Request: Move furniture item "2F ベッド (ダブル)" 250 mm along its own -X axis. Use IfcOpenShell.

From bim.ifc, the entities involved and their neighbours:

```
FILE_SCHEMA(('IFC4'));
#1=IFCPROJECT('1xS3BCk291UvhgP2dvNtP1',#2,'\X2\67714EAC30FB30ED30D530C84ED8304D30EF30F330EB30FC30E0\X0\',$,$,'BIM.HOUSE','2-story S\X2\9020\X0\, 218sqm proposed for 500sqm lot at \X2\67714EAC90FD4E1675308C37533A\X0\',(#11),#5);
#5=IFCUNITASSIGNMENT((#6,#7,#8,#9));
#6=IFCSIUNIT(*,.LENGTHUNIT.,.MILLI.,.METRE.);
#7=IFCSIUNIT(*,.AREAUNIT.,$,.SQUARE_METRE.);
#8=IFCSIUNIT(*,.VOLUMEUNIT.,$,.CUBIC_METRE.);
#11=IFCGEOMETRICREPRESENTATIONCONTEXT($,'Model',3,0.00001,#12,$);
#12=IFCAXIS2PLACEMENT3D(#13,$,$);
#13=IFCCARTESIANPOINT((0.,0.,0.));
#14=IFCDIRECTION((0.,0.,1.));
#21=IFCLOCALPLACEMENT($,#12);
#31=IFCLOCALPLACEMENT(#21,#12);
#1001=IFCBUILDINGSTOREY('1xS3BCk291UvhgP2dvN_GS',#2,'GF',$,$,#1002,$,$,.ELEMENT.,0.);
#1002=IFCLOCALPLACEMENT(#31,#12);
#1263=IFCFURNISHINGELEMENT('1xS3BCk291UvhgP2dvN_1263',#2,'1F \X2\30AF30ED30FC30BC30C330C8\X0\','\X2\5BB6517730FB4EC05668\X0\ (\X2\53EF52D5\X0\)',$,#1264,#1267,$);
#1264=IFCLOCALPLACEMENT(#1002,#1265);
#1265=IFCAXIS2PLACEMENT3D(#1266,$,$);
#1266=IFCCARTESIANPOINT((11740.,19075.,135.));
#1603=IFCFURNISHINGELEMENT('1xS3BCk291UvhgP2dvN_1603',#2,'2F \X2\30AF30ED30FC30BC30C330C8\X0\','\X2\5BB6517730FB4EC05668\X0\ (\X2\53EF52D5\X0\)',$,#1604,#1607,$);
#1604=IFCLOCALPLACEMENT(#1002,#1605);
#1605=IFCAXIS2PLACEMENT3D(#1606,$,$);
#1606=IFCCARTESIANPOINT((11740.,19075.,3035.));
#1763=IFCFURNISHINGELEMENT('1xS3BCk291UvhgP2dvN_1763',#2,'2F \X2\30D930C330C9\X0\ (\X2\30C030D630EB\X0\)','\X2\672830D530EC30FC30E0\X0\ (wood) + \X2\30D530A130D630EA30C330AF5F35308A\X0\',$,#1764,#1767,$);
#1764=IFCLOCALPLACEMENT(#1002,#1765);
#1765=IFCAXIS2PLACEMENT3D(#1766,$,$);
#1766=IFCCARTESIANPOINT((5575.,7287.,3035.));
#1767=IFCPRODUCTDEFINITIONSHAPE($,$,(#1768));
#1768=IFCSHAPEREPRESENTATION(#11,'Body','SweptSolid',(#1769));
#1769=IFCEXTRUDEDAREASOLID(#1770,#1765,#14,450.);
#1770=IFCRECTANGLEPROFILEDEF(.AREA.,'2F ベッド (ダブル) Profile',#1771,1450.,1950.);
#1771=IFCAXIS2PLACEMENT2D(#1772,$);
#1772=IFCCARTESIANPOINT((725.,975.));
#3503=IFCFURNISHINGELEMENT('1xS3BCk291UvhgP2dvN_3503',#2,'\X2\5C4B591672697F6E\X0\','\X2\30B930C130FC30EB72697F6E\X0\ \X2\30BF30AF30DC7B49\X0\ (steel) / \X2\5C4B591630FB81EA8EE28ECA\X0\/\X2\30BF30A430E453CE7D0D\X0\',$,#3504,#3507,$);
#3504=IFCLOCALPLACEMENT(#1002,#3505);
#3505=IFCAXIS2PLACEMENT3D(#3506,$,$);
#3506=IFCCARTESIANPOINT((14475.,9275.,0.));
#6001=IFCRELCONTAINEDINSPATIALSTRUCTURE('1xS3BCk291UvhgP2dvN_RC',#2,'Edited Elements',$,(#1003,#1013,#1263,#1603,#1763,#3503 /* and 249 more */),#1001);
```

```python
import ifcopenshell
import ifcopenshell.api.geometry
import ifcopenshell.util.placement
import ifcopenshell.util.unit

model = ifcopenshell.open("bim.ifc")
unit_scale = ifcopenshell.util.unit.calculate_unit_scale(model)

item = model.by_id(1763)
matrix = ifcopenshell.util.placement.get_local_placement(item.ObjectPlacement)
matrix[:3, 3] -= matrix[:3, 0] * 0.25 / unit_scale
ifcopenshell.api.geometry.edit_object_placement(model, product=item, matrix=matrix, is_si=False)

print(ifcopenshell.util.placement.get_local_placement(item.ObjectPlacement).round(3) + 0.0)

model.write("bim_rev.ifc")
```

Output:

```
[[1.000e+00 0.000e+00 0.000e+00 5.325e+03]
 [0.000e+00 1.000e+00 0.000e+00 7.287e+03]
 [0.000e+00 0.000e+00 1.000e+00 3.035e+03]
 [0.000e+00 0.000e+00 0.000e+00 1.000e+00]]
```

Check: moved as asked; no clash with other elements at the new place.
